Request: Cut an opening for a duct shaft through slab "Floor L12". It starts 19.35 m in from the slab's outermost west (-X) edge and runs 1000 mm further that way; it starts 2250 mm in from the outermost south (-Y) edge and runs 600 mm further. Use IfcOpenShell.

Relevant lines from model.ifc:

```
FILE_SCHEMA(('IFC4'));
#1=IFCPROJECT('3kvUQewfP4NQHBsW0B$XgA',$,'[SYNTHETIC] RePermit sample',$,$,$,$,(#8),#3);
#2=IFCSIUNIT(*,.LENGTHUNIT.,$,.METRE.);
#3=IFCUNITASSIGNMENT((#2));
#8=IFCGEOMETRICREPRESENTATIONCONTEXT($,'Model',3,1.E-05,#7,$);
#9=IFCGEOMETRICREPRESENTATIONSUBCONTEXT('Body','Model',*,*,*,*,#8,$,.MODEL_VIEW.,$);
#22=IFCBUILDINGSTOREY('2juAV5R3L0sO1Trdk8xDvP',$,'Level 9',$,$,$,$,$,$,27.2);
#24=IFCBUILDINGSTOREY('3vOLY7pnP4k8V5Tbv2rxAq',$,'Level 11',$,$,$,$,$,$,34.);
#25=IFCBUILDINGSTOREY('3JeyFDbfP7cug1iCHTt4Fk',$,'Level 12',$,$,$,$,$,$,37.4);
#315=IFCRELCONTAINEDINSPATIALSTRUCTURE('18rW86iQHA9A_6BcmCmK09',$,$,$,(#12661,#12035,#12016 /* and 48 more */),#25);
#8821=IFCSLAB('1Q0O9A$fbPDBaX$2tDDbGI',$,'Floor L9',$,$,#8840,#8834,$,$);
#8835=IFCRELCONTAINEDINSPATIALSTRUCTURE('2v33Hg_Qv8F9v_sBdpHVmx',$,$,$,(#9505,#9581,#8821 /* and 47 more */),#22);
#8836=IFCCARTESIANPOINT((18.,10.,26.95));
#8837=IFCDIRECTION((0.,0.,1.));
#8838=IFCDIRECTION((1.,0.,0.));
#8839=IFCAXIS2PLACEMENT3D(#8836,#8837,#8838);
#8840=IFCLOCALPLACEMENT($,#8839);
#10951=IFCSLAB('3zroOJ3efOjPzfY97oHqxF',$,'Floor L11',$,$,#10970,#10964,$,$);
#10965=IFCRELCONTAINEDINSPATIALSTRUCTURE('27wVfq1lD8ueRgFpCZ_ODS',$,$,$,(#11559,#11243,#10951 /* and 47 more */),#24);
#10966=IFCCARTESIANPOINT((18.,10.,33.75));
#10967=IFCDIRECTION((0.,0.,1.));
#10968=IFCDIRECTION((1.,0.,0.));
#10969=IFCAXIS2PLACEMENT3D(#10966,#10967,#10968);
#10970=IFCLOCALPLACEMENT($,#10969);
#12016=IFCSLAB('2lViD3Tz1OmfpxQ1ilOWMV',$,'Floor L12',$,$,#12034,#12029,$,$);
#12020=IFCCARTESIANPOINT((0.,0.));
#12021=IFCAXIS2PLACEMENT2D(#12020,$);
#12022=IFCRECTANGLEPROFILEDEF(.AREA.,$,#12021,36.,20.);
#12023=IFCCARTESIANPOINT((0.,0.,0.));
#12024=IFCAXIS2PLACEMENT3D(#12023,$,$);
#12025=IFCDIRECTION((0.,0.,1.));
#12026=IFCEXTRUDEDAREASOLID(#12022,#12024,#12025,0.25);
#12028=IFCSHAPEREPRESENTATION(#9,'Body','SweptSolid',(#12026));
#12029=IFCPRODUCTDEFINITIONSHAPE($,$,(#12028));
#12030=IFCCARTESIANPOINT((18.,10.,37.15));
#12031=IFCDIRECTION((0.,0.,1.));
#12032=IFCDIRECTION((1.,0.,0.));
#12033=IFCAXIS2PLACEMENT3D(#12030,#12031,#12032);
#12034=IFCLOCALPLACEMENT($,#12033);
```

```python
import numpy as np
import ifcopenshell
import ifcopenshell.api.feature
import ifcopenshell.api.geometry
import ifcopenshell.api.root
import ifcopenshell.geom
import ifcopenshell.util.placement
import ifcopenshell.util.representation
import ifcopenshell.util.shape
import ifcopenshell.util.unit

model = ifcopenshell.open("model.ifc")
unit_scale = ifcopenshell.util.unit.calculate_unit_scale(model)
settings = ifcopenshell.geom.settings()


def volume(element):
    """Net volume in cubic metres, openings subtracted."""
    shape = ifcopenshell.geom.create_shape(settings, element)
    return ifcopenshell.util.shape.get_volume(shape.geometry)


slab = model.by_guid("2lViD3Tz1OmfpxQ1ilOWMV")
before = volume(slab)

# Extent in the slab's own axes, in metres. The edges named are its -X and -Y sides.
slab_shape = ifcopenshell.geom.create_shape(settings, slab)
vertices = ifcopenshell.util.shape.get_vertices(slab_shape.geometry)
x_min, y_min, bottom = vertices.min(axis=0)
top = vertices[:, 2].max()

opening = ifcopenshell.api.root.create_entity(model, ifc_class="IfcOpeningElement", name="Duct shaft opening", predefined_type="OPENING")
context = ifcopenshell.util.representation.get_context(model, "Model", "Body", "MODEL_VIEW")
width, depth = 1, 0.6
outline = [(0.0, 0.0), (width, 0.0), (width, depth), (0.0, depth), (0.0, 0.0)]
# Overshoot both faces by 50 mm so the cut is clean.
shape = ifcopenshell.api.geometry.add_slab_representation(
    model, context=context, depth=top - bottom + 0.1, polyline=outline
)
ifcopenshell.api.geometry.assign_representation(model, product=opening, representation=shape)

matrix = ifcopenshell.util.placement.get_local_placement(slab.ObjectPlacement)
matrix[:, 3] = matrix @ np.append(np.array([x_min + 19.35, y_min + 2.25, bottom - 0.05]) / unit_scale, 1.0)
ifcopenshell.api.geometry.edit_object_placement(model, product=opening, matrix=matrix, is_si=False)
ifcopenshell.api.feature.add_feature(model, feature=opening, element=slab)

after = volume(slab)

print(f"slab volume {before:.3f} -> {after:.3f} m3")

model.write("model-out.ifc")
```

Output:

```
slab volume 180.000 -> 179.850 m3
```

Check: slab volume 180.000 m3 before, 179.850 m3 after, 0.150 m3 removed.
